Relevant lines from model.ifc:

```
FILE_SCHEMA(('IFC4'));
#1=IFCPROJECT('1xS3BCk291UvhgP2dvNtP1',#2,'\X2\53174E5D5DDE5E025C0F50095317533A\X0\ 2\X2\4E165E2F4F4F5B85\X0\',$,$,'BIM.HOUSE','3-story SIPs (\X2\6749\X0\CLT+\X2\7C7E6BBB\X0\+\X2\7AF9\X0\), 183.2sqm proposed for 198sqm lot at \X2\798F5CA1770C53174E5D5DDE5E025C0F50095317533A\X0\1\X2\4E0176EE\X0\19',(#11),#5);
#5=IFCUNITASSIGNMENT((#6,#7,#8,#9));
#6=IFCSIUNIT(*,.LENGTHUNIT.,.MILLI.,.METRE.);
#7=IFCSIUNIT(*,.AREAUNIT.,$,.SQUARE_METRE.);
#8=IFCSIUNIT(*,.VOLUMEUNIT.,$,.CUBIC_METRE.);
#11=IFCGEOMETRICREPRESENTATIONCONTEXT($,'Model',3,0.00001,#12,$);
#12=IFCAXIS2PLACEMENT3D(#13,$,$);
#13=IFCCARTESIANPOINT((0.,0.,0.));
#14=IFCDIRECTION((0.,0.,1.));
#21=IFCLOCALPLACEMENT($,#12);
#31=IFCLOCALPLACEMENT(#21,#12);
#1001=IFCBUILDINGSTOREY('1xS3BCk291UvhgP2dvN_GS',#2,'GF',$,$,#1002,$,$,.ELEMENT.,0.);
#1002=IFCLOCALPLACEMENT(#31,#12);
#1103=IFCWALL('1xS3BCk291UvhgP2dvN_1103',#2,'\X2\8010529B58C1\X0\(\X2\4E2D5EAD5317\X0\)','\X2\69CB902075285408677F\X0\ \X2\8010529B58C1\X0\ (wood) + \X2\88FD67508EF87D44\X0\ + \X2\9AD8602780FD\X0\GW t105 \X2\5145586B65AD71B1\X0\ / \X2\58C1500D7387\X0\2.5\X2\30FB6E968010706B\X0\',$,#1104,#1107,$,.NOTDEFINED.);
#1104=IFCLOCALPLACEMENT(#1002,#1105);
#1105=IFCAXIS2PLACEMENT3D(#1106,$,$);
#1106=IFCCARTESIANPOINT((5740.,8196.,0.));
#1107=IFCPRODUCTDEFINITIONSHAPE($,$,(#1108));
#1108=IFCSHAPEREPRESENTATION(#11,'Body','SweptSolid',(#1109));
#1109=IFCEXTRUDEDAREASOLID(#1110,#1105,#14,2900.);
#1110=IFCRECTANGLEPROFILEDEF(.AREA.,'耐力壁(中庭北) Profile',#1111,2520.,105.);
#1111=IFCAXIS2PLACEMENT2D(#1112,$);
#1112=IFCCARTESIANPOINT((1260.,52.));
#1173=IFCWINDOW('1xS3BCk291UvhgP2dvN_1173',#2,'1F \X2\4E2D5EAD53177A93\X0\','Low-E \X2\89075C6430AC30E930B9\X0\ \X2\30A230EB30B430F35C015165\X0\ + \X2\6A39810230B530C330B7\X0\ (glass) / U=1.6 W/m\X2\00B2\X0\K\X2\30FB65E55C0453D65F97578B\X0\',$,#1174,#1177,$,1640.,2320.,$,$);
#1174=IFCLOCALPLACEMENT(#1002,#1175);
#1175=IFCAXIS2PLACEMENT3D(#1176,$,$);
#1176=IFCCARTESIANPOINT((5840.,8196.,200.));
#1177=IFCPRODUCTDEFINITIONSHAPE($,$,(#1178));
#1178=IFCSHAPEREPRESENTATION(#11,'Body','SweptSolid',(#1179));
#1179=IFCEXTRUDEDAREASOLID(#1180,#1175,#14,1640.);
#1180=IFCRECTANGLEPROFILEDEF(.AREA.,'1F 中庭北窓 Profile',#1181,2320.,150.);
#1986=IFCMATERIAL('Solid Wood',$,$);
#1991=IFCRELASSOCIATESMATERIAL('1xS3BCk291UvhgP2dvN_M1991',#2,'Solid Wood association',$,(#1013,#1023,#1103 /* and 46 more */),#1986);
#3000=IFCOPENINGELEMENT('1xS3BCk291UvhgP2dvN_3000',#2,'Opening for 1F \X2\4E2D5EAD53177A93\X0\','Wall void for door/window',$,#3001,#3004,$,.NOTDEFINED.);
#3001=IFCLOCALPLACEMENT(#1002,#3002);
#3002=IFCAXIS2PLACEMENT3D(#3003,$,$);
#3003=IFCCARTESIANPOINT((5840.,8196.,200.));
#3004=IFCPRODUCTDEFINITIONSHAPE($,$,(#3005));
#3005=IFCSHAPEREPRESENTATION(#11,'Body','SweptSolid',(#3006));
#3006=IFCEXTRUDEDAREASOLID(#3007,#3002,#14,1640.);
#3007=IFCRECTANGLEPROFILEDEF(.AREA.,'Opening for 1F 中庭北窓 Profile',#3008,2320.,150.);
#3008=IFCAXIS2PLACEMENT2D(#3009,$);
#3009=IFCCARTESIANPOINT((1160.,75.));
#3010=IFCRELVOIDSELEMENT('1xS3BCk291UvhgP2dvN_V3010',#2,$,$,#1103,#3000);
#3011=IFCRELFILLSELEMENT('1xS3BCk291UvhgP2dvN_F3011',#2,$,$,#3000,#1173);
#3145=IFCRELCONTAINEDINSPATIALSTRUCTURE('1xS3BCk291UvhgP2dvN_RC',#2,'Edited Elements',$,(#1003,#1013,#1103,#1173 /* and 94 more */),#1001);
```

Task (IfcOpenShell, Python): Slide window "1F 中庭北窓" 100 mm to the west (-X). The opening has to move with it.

```python
import ifcopenshell
import ifcopenshell.api.geometry
import ifcopenshell.util.placement
import ifcopenshell.util.unit

model = ifcopenshell.open("model.ifc")
unit_scale = ifcopenshell.util.unit.calculate_unit_scale(model)

window = model.by_id(1173)
opening = window.FillsVoids[0].RelatingOpeningElement
wall = opening.VoidsElements[0].RelatingBuildingElement

wall_matrix = ifcopenshell.util.placement.get_local_placement(wall.ObjectPlacement)
shift = wall_matrix[:3, 0] * -0.1 / unit_scale
before = ifcopenshell.util.placement.get_local_placement(window.ObjectPlacement)[:3, 3].copy()

# The window is not placed relative to its opening, so move both.
for product in (opening, window):
    matrix = ifcopenshell.util.placement.get_local_placement(product.ObjectPlacement)
    matrix[:3, 3] += shift
    ifcopenshell.api.geometry.edit_object_placement(model, product=product, matrix=matrix, is_si=False)

after = ifcopenshell.util.placement.get_local_placement(window.ObjectPlacement)[:3, 3]
print("window moved by", (after - before).round(3) + 0.0)

model.write("model-out.ifc")
```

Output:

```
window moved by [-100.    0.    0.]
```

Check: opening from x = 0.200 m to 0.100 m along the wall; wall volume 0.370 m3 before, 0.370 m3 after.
